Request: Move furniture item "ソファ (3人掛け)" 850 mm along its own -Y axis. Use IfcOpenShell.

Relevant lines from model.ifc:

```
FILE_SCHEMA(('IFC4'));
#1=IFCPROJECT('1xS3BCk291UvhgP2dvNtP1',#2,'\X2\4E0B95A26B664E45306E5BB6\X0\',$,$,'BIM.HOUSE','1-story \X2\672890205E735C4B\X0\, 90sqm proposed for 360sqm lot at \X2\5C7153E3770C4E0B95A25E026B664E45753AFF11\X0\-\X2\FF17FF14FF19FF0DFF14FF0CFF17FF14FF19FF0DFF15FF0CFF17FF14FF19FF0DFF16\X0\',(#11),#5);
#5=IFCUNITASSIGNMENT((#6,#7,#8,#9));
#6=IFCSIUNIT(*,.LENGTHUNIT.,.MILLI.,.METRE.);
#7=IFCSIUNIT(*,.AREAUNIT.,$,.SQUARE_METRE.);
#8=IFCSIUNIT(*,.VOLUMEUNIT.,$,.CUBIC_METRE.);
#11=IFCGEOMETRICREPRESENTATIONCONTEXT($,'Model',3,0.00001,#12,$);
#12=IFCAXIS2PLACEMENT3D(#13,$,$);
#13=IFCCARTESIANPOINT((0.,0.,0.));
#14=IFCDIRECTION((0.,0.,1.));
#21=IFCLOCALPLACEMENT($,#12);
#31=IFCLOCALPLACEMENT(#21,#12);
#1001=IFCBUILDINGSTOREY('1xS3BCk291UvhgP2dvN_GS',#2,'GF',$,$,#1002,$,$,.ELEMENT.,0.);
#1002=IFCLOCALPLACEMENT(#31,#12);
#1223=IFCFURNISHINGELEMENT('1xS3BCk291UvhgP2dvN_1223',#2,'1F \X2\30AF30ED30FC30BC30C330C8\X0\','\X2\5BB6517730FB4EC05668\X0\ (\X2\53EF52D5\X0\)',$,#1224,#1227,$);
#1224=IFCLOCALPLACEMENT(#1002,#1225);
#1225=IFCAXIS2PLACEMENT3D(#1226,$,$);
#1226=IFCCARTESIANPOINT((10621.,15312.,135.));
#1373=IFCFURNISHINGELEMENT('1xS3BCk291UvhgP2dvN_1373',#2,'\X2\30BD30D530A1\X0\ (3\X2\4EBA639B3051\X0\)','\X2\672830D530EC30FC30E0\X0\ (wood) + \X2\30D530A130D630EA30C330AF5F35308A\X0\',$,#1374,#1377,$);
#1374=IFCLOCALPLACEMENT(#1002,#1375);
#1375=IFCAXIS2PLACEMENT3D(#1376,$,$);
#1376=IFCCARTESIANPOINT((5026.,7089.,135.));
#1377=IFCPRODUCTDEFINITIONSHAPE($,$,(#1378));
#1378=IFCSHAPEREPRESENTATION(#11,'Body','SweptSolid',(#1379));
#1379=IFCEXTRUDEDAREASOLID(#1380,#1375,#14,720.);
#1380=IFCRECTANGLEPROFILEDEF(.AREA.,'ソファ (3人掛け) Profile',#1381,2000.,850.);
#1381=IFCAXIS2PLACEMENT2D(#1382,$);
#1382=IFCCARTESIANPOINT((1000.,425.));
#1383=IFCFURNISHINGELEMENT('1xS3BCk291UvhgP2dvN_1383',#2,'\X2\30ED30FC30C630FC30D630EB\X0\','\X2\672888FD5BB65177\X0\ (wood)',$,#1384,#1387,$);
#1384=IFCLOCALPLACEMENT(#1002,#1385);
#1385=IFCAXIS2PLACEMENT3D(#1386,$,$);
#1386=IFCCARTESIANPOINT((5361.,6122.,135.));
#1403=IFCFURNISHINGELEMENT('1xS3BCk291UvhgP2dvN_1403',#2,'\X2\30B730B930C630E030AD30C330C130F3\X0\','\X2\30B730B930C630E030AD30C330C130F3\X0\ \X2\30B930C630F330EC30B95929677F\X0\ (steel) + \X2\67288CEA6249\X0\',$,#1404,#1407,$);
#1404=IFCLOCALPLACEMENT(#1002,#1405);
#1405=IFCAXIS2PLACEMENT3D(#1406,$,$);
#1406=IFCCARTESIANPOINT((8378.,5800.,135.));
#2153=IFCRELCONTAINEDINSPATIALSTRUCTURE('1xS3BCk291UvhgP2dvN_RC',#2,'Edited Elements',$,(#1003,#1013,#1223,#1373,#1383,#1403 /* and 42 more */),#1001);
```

```python
import ifcopenshell
import ifcopenshell.api.geometry
import ifcopenshell.util.placement

model = ifcopenshell.open("model.ifc")

item = model.by_guid("1xS3BCk291UvhgP2dvN_1373")
matrix = ifcopenshell.util.placement.get_local_placement(item.ObjectPlacement)
matrix[:3, 3] -= matrix[:3, 1] * 850.0
ifcopenshell.api.geometry.edit_object_placement(model, product=item, matrix=matrix, is_si=False)

print(ifcopenshell.util.placement.get_local_placement(item.ObjectPlacement).round(3) + 0.0)

model.write("model_updated.ifc")
```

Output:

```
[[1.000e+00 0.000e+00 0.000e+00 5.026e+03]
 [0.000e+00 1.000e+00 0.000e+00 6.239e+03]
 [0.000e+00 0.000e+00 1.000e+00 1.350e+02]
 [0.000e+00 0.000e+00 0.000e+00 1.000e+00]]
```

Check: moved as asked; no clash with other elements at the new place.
